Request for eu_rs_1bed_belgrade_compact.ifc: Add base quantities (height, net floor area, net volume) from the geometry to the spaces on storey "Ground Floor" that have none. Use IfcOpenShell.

First a look at what the model holds.

```python
import ifcopenshell
import ifcopenshell.util.element
import ifcopenshell.util.unit

model = ifcopenshell.open("eu_rs_1bed_belgrade_compact.ifc")
print(model.schema)
for unit_type in ("LENGTHUNIT", "AREAUNIT", "VOLUMEUNIT"):
    print(unit_type, ifcopenshell.util.unit.calculate_unit_scale(model, unit_type))
storey = next(s for s in model.by_type("IfcBuildingStorey") if s.Name == "Ground Floor")
spaces = [e for e in ifcopenshell.util.element.get_decomposition(storey) if e.is_a("IfcSpace")]
for e in sorted(spaces, key=lambda e: e.id()):
    print(e.id(), e.is_a(), e.Name, list(ifcopenshell.util.element.get_psets(e, qtos_only=True)), sep=" | ")
```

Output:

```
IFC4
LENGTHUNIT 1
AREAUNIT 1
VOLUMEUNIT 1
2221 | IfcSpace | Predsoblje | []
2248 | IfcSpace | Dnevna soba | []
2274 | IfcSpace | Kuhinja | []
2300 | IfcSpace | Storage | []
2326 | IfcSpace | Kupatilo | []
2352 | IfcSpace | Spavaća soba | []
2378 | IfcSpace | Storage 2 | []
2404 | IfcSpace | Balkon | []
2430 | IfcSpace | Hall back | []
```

```python
import ifcopenshell
import ifcopenshell.api.pset
import ifcopenshell.geom
import ifcopenshell.util.element
import ifcopenshell.util.shape
import ifcopenshell.util.unit

model = ifcopenshell.open("eu_rs_1bed_belgrade_compact.ifc")
unit_scale = ifcopenshell.util.unit.calculate_unit_scale(model)
area_scale = ifcopenshell.util.unit.calculate_unit_scale(model, "AREAUNIT")
volume_scale = ifcopenshell.util.unit.calculate_unit_scale(model, "VOLUMEUNIT")
settings = ifcopenshell.geom.settings()

storey = next(s for s in model.by_type("IfcBuildingStorey") if s.Name == "Ground Floor")
spaces = [e for e in ifcopenshell.util.element.get_decomposition(storey) if e.is_a("IfcSpace")]

for e in sorted(spaces, key=lambda e: e.id()):
    if ifcopenshell.util.element.get_psets(e, qtos_only=True, should_inherit=False):
        continue
    # Geometry comes back in metres, in the element's own axes.
    shape = ifcopenshell.geom.create_shape(settings, e)
    values = {
        "Height": ifcopenshell.util.shape.get_z(shape.geometry) / unit_scale,
        "NetFloorArea": ifcopenshell.util.shape.get_footprint_area(shape.geometry) / area_scale,
        "NetVolume": ifcopenshell.util.shape.get_volume(shape.geometry) / volume_scale,
    }
    qto = ifcopenshell.api.pset.add_qto(model, product=e, name="Qto_SpaceBaseQuantities")
    ifcopenshell.api.pset.edit_qto(model, qto=qto, properties=values)
    print(e.id(), {k: round(v, 3) for k, v in values.items()})

model.write("eu_rs_1bed_belgrade_compact_rev.ifc")
```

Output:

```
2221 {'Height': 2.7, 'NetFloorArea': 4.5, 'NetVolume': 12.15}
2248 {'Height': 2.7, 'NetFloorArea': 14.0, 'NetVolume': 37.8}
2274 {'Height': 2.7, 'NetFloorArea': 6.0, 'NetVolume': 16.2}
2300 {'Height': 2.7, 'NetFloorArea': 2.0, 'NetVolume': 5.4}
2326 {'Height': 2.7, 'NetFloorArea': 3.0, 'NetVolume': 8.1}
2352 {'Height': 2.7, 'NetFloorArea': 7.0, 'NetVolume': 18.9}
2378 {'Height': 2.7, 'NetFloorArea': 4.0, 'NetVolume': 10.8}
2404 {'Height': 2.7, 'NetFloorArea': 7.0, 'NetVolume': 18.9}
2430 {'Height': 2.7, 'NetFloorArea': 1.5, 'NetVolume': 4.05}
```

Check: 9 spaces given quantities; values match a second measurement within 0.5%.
